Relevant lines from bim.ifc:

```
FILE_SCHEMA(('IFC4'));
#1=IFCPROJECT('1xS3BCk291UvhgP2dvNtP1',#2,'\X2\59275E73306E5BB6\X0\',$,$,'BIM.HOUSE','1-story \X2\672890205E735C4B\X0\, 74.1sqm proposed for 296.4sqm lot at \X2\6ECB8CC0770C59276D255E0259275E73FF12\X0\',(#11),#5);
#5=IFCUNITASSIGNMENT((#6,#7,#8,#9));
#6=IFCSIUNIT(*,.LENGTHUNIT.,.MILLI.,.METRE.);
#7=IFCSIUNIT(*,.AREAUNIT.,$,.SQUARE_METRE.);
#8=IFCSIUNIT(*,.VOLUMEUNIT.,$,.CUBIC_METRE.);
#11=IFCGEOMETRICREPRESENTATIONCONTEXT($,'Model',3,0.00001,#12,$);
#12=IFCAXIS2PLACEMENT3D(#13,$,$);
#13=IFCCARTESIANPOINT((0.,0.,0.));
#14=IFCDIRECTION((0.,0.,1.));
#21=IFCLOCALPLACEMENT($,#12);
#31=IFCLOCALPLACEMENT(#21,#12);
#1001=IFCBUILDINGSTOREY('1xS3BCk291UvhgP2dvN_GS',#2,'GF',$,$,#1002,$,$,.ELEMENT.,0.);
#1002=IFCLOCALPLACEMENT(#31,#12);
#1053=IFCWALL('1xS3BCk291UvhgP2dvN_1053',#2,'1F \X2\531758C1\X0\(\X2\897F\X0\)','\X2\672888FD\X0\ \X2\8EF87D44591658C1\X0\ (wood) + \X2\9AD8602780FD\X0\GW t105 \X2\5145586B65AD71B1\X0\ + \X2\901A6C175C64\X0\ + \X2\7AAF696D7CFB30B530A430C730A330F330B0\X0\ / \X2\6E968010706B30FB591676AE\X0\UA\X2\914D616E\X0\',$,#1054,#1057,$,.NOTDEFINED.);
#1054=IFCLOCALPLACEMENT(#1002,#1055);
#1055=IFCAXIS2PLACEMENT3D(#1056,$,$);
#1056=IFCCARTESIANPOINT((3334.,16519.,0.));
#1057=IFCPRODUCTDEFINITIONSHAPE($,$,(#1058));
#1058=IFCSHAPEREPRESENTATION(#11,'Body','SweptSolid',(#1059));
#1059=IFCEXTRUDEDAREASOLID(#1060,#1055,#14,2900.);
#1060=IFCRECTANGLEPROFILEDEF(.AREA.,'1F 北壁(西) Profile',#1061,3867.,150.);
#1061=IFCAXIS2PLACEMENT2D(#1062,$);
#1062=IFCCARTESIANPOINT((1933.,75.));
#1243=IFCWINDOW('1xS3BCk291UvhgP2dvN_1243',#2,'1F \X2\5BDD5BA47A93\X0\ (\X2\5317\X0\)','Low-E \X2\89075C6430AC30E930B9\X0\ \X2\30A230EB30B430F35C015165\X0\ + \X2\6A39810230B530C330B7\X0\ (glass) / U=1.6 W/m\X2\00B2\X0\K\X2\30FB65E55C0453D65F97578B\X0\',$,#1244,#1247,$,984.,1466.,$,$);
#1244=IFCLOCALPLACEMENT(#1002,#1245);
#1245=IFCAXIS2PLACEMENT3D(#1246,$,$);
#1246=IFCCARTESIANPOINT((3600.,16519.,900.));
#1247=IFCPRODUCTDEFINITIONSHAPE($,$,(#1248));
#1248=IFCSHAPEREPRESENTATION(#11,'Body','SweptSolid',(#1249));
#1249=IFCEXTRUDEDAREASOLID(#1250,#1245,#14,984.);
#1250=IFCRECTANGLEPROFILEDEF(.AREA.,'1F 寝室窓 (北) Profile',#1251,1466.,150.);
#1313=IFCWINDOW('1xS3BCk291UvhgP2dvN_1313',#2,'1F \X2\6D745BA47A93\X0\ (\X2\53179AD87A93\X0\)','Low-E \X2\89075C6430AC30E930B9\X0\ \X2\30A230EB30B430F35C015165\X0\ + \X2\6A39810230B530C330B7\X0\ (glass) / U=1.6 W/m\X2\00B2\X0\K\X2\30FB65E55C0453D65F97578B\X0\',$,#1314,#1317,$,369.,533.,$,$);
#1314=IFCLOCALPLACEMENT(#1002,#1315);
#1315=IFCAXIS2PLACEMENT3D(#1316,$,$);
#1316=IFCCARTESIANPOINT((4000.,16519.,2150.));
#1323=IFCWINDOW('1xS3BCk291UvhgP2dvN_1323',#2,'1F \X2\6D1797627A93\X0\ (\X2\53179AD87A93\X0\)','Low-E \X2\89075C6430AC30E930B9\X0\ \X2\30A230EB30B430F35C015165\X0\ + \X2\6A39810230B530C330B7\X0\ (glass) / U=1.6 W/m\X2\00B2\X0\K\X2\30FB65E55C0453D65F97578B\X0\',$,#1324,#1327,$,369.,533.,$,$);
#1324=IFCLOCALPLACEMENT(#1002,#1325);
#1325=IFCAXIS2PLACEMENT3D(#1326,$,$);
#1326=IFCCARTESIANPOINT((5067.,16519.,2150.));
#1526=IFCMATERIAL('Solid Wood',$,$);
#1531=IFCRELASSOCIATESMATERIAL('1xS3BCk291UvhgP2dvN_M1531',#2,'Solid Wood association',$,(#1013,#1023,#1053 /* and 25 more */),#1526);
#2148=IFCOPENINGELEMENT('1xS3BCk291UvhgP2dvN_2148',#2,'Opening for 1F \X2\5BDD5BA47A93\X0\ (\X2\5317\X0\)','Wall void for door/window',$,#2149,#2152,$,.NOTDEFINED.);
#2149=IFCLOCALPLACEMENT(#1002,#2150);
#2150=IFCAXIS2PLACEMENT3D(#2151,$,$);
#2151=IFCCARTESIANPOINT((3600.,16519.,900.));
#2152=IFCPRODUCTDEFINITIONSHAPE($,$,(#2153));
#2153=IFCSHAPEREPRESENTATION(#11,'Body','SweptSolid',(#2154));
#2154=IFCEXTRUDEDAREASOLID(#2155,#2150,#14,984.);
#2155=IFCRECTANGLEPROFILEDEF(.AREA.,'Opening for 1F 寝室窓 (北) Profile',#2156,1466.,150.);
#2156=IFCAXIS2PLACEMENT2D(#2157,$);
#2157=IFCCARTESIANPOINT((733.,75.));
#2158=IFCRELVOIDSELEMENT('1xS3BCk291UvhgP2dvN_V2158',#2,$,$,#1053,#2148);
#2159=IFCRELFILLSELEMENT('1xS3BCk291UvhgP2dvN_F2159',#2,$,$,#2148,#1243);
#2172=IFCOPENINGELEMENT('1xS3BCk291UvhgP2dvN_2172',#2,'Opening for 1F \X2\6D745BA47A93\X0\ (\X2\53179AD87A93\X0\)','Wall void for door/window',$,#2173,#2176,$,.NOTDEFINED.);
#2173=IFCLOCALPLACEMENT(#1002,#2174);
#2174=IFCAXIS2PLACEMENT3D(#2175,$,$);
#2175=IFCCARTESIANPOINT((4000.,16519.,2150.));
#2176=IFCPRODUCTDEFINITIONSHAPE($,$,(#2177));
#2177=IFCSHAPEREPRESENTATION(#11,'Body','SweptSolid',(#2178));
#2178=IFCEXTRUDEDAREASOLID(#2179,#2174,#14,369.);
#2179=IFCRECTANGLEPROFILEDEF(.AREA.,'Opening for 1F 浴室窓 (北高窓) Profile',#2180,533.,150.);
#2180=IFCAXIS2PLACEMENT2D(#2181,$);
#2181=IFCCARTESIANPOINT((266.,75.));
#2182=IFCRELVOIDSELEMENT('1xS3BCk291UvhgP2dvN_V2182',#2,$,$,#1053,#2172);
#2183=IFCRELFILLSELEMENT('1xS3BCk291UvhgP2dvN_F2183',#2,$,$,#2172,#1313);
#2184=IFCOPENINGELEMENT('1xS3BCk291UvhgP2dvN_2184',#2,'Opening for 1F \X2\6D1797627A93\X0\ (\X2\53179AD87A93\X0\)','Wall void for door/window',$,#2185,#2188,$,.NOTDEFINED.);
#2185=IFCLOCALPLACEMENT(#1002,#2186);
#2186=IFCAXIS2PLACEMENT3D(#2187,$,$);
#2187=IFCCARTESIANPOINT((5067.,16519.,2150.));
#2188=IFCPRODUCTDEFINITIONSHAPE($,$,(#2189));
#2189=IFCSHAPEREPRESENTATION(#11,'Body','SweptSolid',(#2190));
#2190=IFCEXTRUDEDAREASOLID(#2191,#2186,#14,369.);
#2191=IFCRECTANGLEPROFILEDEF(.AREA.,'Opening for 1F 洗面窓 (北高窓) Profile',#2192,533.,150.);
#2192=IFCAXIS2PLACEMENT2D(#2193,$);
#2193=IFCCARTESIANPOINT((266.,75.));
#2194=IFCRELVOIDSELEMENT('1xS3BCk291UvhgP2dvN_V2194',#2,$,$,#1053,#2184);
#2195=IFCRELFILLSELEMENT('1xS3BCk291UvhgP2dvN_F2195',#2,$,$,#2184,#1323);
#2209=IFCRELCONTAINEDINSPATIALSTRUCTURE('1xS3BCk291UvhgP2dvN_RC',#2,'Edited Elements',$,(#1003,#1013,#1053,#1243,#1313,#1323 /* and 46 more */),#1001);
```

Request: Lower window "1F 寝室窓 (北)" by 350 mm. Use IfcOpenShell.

```python
import numpy as np
import ifcopenshell
import ifcopenshell.api.geometry
import ifcopenshell.util.placement
import ifcopenshell.util.unit

model = ifcopenshell.open("bim.ifc")
unit_scale = ifcopenshell.util.unit.calculate_unit_scale(model)

window = model.by_guid("1xS3BCk291UvhgP2dvN_1243")
opening = window.FillsVoids[0].RelatingOpeningElement
dz = -0.35 / unit_scale

shift = np.array([0.0, 0.0, dz])
# The window is not placed relative to its opening, so move both.
for product in (opening, window):
    matrix = ifcopenshell.util.placement.get_local_placement(product.ObjectPlacement)
    matrix[:3, 3] += shift
    ifcopenshell.api.geometry.edit_object_placement(model, product=product, matrix=matrix, is_si=False)

print(f"moved by {dz * unit_scale:+.3f} m")

model.write("bim-out.ifc")
```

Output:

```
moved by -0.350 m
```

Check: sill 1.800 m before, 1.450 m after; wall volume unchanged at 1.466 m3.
